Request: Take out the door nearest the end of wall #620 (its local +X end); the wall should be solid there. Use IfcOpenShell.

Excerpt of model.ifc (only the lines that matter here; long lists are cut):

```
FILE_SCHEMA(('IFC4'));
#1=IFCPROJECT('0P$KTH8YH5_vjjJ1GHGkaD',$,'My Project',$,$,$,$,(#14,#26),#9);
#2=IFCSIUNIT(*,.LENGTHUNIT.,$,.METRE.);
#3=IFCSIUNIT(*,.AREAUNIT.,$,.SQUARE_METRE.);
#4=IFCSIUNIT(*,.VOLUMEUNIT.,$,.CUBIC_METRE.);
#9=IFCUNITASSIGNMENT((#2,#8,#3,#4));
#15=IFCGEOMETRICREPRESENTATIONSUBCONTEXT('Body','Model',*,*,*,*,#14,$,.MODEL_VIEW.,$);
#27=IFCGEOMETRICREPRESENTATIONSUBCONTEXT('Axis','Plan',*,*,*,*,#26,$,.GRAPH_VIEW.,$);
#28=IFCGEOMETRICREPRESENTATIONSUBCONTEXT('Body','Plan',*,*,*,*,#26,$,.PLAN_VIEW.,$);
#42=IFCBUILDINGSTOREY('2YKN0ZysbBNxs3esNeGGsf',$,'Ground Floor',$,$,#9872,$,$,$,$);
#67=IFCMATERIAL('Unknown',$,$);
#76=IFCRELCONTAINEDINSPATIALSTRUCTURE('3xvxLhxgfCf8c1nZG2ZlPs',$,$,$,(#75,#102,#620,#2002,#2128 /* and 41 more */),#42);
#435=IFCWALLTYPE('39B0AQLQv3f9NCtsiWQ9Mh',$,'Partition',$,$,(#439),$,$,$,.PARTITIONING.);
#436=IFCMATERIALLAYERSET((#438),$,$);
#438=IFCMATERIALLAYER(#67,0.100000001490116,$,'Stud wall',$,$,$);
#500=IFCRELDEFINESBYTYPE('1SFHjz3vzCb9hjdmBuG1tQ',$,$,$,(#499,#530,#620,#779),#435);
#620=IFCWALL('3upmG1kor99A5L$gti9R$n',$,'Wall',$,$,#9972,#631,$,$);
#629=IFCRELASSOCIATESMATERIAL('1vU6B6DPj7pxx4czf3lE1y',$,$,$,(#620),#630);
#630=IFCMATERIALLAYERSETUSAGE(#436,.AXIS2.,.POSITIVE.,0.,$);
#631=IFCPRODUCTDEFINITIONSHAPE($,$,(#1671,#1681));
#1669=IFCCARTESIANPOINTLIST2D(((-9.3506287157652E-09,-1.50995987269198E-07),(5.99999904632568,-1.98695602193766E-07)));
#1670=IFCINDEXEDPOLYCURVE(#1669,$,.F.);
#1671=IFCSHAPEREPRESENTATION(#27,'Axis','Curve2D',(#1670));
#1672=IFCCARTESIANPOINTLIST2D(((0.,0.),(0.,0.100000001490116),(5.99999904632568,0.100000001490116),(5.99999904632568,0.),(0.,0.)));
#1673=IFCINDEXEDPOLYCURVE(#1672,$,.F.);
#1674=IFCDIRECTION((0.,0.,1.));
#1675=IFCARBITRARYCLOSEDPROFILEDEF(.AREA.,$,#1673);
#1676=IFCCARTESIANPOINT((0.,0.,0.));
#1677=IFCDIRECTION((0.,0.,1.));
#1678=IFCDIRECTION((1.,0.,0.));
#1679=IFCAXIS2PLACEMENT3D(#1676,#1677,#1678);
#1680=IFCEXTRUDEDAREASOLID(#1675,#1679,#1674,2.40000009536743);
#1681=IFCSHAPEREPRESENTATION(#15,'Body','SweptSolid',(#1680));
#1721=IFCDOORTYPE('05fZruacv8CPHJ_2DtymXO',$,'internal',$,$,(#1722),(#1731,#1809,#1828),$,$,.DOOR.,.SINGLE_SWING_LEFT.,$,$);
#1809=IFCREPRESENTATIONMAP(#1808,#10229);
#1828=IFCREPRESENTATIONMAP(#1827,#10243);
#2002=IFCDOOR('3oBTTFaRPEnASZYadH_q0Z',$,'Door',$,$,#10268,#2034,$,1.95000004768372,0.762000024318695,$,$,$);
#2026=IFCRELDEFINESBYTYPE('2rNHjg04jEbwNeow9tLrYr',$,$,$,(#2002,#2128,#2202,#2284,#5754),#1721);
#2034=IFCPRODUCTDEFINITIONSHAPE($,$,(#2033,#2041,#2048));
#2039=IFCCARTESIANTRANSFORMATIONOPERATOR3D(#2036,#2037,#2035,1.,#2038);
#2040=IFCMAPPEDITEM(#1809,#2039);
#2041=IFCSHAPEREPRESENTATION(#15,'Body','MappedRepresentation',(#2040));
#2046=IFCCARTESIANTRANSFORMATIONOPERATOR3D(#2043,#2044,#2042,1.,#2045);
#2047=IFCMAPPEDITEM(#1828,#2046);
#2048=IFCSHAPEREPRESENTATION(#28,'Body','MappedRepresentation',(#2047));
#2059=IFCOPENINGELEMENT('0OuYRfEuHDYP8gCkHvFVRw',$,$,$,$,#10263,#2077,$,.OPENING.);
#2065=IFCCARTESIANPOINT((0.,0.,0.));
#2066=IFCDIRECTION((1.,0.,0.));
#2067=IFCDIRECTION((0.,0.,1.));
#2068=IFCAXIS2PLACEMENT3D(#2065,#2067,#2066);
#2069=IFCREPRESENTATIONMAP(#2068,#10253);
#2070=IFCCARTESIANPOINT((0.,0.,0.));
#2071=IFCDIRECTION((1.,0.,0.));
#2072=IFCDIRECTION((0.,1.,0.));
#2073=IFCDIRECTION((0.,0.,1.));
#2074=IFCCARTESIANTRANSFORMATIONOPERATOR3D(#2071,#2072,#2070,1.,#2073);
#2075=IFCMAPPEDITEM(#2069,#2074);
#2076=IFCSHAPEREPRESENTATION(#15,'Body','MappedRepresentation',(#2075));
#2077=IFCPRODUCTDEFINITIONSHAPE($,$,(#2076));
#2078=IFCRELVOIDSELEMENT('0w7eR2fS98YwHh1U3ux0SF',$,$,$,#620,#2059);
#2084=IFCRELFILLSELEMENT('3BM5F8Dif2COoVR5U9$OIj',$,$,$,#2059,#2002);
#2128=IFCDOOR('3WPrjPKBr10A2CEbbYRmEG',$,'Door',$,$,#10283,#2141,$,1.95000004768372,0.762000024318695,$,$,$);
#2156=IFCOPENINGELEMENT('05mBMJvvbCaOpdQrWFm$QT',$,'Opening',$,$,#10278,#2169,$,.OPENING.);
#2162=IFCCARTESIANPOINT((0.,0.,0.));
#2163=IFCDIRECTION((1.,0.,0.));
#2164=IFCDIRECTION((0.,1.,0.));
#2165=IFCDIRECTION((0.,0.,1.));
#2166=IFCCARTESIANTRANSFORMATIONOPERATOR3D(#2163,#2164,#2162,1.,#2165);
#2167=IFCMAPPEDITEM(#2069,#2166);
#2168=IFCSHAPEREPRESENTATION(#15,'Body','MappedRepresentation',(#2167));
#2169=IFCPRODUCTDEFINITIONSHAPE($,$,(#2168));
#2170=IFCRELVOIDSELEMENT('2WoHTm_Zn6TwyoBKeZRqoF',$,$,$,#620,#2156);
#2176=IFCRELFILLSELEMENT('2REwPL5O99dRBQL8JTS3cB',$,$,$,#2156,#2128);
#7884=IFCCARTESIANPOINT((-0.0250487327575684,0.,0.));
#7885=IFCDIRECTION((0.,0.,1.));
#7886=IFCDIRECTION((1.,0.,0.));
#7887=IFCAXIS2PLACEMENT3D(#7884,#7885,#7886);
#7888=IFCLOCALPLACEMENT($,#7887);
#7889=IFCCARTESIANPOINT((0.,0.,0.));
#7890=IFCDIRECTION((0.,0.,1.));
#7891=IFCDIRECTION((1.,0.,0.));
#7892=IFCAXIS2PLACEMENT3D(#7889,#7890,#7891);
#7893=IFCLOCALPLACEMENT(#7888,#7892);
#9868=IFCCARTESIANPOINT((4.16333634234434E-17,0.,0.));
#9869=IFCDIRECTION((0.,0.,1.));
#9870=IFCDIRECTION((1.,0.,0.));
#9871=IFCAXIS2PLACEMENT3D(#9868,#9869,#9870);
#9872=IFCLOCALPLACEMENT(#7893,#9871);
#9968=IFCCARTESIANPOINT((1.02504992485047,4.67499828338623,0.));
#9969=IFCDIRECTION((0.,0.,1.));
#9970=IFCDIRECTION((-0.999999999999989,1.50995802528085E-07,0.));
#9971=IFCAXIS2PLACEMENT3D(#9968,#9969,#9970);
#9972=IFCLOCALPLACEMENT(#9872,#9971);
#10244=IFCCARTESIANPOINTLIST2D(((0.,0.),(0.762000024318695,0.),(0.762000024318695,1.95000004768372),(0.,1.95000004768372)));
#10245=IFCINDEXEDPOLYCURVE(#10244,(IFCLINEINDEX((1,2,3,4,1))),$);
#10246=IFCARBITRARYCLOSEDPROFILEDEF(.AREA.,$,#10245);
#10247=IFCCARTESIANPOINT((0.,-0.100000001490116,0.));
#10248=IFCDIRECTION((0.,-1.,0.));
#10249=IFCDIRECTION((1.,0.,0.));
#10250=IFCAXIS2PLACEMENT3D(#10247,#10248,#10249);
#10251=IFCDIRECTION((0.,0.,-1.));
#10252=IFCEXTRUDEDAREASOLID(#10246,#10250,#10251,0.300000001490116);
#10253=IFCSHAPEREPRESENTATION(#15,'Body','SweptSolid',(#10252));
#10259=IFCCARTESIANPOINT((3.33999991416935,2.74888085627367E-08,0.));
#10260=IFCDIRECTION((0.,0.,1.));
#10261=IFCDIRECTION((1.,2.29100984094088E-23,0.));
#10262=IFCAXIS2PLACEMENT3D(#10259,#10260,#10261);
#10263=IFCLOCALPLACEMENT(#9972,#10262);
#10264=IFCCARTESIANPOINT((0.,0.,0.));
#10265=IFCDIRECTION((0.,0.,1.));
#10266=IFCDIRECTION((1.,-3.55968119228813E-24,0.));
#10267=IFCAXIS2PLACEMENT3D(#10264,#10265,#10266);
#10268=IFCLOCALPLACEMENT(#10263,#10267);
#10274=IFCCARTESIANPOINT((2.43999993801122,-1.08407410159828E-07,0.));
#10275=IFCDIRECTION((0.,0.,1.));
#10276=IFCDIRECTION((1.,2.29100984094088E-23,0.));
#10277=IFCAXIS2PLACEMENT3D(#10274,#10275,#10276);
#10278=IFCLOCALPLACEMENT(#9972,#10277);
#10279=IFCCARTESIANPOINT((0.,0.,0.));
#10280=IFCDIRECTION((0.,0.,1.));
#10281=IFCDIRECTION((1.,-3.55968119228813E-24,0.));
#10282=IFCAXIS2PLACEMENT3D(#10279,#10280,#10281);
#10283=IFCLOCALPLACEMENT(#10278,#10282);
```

```python
import ifcopenshell
import ifcopenshell.api.feature
import ifcopenshell.api.root
import ifcopenshell.geom
import ifcopenshell.util.shape

model = ifcopenshell.open("model.ifc")
settings = ifcopenshell.geom.settings()


def volume(element):
    """Net volume in cubic metres, openings subtracted."""
    shape = ifcopenshell.geom.create_shape(settings, element)
    return ifcopenshell.util.shape.get_volume(shape.geometry)


door = model.by_guid("3oBTTFaRPEnASZYadH_q0Z")
opening = door.FillsVoids[0].RelatingOpeningElement
wall = opening.VoidsElements[0].RelatingBuildingElement
before = volume(wall)

ifcopenshell.api.root.remove_product(model, product=door)
ifcopenshell.api.feature.remove_feature(model, feature=opening)

after = volume(wall)

print(f"wall volume {before:.3f} -> {after:.3f} m3")

model.write("model_rev.ifc")
```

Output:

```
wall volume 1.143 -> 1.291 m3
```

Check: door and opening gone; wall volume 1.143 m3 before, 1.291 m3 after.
